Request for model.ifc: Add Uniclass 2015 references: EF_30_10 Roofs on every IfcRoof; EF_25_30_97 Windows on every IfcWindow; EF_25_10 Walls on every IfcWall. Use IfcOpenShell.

First a look at what the model holds.

```python
import ifcopenshell

model = ifcopenshell.open("model.ifc")
print(model.schema)
print("classifications:", [c.Name for c in model.by_type("IfcClassification")])
for ifc_class in ("IfcDoor", "IfcRoof", "IfcStair", "IfcWall", "IfcWindow"):
    print(ifc_class, len(model.by_type(ifc_class)))
```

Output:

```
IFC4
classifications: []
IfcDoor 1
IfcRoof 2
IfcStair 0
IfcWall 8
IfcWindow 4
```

```python
import ifcopenshell
import ifcopenshell.api.classification

model = ifcopenshell.open("model.ifc")

system = ifcopenshell.api.classification.add_classification(model, classification="Uniclass 2015")

codes = {
    "IfcRoof": ("EF_30_10", "Roofs"),
    "IfcWindow": ("EF_25_30_97", "Windows"),
    "IfcWall": ("EF_25_10", "Walls"),
}
for ifc_class, (code, name) in codes.items():
    products = model.by_type(ifc_class)
    ifcopenshell.api.classification.add_reference(
        model, products=products, classification=system, identification=code, name=name
    )
    print(code, len(products))

model.write("model_rev.ifc")
```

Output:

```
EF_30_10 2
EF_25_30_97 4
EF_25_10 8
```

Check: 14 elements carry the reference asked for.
